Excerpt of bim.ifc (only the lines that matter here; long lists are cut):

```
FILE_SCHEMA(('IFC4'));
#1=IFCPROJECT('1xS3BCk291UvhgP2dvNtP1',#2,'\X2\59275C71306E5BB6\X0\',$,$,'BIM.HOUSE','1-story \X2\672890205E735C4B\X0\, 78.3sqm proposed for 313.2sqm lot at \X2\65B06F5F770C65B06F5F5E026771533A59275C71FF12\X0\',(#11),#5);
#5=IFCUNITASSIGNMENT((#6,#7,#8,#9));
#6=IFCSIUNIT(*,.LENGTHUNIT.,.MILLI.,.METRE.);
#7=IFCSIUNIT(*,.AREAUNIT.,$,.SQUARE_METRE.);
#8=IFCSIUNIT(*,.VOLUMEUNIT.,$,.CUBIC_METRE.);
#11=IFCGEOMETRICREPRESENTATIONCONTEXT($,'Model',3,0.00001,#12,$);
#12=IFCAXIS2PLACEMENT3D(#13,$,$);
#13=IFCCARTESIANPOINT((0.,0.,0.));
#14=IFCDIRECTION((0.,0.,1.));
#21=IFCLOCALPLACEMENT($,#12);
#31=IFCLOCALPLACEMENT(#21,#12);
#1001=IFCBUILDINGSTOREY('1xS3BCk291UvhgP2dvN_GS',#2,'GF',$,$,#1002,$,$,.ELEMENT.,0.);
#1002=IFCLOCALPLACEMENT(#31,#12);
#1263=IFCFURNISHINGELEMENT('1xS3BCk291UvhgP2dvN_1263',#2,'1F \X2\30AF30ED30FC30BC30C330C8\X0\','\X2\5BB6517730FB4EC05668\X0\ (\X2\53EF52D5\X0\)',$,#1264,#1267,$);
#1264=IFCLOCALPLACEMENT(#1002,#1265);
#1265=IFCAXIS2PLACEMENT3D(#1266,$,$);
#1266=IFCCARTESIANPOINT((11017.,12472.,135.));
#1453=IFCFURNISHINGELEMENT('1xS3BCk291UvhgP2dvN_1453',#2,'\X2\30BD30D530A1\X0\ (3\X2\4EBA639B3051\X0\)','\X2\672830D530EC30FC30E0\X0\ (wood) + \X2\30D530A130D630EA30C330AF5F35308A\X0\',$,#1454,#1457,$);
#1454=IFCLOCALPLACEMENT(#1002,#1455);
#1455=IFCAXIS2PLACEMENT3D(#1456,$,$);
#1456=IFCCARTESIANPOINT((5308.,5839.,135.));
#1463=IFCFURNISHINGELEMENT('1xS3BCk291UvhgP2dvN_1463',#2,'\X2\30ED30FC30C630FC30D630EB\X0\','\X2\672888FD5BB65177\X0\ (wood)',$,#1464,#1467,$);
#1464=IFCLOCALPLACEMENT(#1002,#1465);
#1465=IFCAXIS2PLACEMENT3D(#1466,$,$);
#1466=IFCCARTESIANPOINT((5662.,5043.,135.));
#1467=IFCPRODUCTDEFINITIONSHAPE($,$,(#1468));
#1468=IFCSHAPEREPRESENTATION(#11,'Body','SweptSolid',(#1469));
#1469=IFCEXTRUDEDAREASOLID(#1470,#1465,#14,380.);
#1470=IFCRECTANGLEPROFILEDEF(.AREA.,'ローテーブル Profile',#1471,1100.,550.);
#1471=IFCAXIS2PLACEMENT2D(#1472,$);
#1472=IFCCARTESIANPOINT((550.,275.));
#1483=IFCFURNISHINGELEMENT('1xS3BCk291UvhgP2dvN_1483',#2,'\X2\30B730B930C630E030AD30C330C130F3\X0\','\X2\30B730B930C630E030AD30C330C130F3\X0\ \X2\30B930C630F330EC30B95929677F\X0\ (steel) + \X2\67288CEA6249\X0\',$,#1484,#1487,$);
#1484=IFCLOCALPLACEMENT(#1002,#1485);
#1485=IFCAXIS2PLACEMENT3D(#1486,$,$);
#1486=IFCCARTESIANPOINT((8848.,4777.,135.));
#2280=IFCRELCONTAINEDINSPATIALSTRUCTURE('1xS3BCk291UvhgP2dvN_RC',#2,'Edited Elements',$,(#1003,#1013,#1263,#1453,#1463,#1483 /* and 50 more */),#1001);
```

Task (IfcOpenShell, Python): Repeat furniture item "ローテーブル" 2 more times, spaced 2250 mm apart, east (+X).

```python
import numpy as np
import ifcopenshell
import ifcopenshell.api.geometry
import ifcopenshell.api.root
import ifcopenshell.util.element
import ifcopenshell.util.placement
import ifcopenshell.util.unit

model = ifcopenshell.open("bim.ifc")
unit_scale = ifcopenshell.util.unit.calculate_unit_scale(model)


def reuse_history(source, copy):
    """copy_class also copies each property set's owner history, people and application; keep the originals."""
    for rel in copy.IsDefinedBy:
        if rel.is_a("IfcRelDefinesByProperties") and (history := rel.RelatingPropertyDefinition.OwnerHistory):
            rel.RelatingPropertyDefinition.OwnerHistory = source.OwnerHistory
            ifcopenshell.util.element.remove_deep2(model, history)


source = model.by_id(1463)
base = ifcopenshell.util.placement.get_local_placement(source.ObjectPlacement)
step = np.array([1.0, 0.0, 0.0]) * 2.25 / unit_scale

for i in range(1, 3):
    copy = ifcopenshell.api.root.copy_class(model, product=source)
    copy.Representation = ifcopenshell.util.element.copy_deep(
        model, source.Representation, exclude=["IfcGeometricRepresentationContext", "IfcRepresentationMap"]
    )
    reuse_history(source, copy)
    matrix = base.copy()
    matrix[:3, 3] += i * step
    print("added at", matrix[:3, 3].round(3) + 0.0)
    ifcopenshell.api.geometry.edit_object_placement(model, product=copy, matrix=matrix, is_si=False)

model.write("bim_rev.ifc")
```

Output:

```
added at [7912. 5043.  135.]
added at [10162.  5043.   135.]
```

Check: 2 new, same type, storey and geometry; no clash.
